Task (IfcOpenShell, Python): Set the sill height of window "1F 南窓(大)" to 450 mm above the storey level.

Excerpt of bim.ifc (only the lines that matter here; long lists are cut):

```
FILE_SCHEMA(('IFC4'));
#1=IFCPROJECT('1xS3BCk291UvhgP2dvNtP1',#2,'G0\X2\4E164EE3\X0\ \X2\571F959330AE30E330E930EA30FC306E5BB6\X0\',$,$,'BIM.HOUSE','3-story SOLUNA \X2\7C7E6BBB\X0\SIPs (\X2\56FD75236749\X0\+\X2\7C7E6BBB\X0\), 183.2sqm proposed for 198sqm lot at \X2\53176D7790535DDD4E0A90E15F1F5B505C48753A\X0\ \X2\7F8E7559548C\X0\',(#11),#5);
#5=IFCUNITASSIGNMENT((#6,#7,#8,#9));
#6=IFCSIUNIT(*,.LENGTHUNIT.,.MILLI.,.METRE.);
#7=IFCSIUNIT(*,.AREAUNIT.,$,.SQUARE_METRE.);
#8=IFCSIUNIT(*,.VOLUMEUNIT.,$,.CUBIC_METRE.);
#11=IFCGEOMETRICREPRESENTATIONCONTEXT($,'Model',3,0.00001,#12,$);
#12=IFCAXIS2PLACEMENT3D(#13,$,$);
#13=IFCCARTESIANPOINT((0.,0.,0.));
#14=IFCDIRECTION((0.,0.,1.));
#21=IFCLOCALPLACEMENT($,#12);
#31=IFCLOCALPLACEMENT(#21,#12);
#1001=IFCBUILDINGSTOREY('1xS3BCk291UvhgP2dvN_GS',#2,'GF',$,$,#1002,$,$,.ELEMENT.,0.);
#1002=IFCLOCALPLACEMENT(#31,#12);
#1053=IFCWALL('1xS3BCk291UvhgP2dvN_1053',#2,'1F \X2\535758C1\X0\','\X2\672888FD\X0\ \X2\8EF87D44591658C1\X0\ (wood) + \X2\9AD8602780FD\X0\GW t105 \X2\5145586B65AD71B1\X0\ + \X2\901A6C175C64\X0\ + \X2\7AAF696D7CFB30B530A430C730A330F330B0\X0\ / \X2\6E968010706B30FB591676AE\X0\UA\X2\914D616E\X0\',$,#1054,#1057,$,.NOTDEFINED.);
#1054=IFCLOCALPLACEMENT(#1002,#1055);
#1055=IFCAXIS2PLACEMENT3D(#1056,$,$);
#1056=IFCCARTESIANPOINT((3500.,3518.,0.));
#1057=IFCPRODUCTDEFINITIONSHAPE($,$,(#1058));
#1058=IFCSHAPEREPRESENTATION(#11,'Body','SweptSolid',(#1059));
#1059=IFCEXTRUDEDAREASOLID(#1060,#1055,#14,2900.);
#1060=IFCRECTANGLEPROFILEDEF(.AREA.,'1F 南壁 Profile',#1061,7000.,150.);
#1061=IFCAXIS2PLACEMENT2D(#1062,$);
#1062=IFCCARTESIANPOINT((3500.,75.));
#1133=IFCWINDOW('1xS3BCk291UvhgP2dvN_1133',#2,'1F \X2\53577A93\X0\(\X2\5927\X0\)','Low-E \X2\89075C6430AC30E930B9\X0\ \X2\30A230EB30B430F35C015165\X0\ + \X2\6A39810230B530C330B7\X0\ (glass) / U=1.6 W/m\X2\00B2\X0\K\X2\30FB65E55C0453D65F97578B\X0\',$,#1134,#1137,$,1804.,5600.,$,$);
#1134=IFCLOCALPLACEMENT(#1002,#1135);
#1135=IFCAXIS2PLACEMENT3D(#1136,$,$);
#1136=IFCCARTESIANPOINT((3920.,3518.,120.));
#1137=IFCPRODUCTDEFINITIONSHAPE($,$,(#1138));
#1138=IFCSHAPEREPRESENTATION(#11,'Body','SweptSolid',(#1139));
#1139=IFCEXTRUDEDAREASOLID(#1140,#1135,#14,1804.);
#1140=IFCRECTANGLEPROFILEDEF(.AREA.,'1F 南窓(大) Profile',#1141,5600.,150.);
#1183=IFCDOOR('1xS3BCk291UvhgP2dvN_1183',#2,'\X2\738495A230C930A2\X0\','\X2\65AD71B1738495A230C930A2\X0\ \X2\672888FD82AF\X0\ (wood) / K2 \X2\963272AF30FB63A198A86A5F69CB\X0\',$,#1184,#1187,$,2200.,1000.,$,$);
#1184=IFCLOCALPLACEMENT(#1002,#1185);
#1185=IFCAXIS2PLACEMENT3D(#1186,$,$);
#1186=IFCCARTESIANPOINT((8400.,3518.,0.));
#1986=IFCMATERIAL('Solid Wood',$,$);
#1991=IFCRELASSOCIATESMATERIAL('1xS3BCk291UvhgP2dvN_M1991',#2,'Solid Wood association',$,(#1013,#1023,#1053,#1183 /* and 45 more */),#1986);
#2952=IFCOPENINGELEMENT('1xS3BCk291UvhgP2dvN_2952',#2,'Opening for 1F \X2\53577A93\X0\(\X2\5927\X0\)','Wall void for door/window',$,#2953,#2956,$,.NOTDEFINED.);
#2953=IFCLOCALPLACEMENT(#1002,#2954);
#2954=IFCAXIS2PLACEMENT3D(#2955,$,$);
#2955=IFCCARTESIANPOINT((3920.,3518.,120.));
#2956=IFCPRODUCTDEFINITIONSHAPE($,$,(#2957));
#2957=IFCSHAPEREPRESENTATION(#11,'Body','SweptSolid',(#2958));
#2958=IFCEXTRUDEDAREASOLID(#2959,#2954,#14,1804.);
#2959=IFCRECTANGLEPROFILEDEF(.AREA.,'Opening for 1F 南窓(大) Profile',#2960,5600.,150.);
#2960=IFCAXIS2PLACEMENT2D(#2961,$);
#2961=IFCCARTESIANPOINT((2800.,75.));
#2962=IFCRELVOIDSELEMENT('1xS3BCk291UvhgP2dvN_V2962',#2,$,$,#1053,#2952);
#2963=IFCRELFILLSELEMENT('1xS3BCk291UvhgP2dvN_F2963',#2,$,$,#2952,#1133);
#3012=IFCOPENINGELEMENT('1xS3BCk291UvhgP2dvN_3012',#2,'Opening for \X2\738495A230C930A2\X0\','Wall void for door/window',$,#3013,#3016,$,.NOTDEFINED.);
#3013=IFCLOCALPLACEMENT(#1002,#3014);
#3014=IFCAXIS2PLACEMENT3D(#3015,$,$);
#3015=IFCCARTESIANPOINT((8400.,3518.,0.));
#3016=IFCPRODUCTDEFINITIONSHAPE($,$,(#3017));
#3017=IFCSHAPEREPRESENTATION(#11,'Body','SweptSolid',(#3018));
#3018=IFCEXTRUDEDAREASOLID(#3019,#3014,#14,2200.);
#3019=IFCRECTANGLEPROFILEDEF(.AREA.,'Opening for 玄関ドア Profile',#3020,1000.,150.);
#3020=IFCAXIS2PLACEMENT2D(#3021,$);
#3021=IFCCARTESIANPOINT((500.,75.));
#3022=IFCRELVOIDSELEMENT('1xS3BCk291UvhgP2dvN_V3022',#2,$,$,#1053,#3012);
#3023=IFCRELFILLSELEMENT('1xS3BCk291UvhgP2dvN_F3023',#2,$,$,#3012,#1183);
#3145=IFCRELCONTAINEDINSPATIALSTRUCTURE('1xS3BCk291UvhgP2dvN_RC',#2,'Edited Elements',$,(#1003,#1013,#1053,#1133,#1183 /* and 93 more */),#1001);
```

```python
import numpy as np
import ifcopenshell
import ifcopenshell.api.geometry
import ifcopenshell.geom
import ifcopenshell.util.element
import ifcopenshell.util.placement
import ifcopenshell.util.shape
import ifcopenshell.util.unit

model = ifcopenshell.open("bim.ifc")
unit_scale = ifcopenshell.util.unit.calculate_unit_scale(model)

window = model.by_id(1133)
opening = window.FillsVoids[0].RelatingOpeningElement
storey = ifcopenshell.util.element.get_container(window, ifc_class="IfcBuildingStorey")
level = ifcopenshell.util.placement.get_local_placement(storey.ObjectPlacement)[2, 3]

# The opening's origin need not be at the sill, so measure its lowest point.
shape = ifcopenshell.geom.create_shape(ifcopenshell.geom.settings(), opening)
bottom = ifcopenshell.util.shape.get_shape_bottom_elevation(shape, shape.geometry) / unit_scale
dz = level + 0.45 / unit_scale - bottom

shift = np.array([0.0, 0.0, dz])
# The window is not placed relative to its opening, so move both.
for product in (opening, window):
    matrix = ifcopenshell.util.placement.get_local_placement(product.ObjectPlacement)
    matrix[:3, 3] += shift
    ifcopenshell.api.geometry.edit_object_placement(model, product=product, matrix=matrix, is_si=False)

print(f"moved by {dz * unit_scale:+.3f} m")

model.write("bim_v2.ifc")
```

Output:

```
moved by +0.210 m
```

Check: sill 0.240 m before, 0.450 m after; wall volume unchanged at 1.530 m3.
